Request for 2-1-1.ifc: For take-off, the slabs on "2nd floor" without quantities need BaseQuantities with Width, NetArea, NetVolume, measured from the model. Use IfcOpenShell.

First a look at what the model holds.

```python
import ifcopenshell
import ifcopenshell.util.element
import ifcopenshell.util.unit

model = ifcopenshell.open("2-1-1.ifc")
print(model.schema)
for unit_type in ("LENGTHUNIT", "AREAUNIT", "VOLUMEUNIT"):
    print(unit_type, ifcopenshell.util.unit.calculate_unit_scale(model, unit_type))
storey = next(s for s in model.by_type("IfcBuildingStorey") if s.Name == "2nd floor")
slabs = [e for e in ifcopenshell.util.element.get_decomposition(storey) if e.is_a("IfcSlab")]
for e in sorted(slabs, key=lambda e: e.id()):
    print(e.id(), e.is_a(), e.Name, list(ifcopenshell.util.element.get_psets(e, qtos_only=True)), sep=" | ")
```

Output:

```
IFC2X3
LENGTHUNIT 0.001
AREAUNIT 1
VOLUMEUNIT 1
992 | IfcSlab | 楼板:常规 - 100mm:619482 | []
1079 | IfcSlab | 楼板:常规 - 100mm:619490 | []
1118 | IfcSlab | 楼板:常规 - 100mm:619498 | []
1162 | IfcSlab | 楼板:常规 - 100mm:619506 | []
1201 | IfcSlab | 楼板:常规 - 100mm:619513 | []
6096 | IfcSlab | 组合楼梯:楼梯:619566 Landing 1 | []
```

```python
import ifcopenshell
import ifcopenshell.api.pset
import ifcopenshell.geom
import ifcopenshell.util.element
import ifcopenshell.util.shape
import ifcopenshell.util.unit

model = ifcopenshell.open("2-1-1.ifc")
unit_scale = ifcopenshell.util.unit.calculate_unit_scale(model)
area_scale = ifcopenshell.util.unit.calculate_unit_scale(model, "AREAUNIT")
volume_scale = ifcopenshell.util.unit.calculate_unit_scale(model, "VOLUMEUNIT")
settings = ifcopenshell.geom.settings()

storey = next(s for s in model.by_type("IfcBuildingStorey") if s.Name == "2nd floor")
slabs = [e for e in ifcopenshell.util.element.get_decomposition(storey) if e.is_a("IfcSlab")]

for e in sorted(slabs, key=lambda e: e.id()):
    if ifcopenshell.util.element.get_psets(e, qtos_only=True, should_inherit=False):
        continue
    # Geometry comes back in metres, in the element's own axes.
    shape = ifcopenshell.geom.create_shape(settings, e)
    values = {
        "Width": ifcopenshell.util.shape.get_z(shape.geometry) / unit_scale,
        "NetArea": ifcopenshell.util.shape.get_footprint_area(shape.geometry) / area_scale,
        "NetVolume": ifcopenshell.util.shape.get_volume(shape.geometry) / volume_scale,
    }
    qto = ifcopenshell.api.pset.add_qto(model, product=e, name="BaseQuantities")
    ifcopenshell.api.pset.edit_qto(model, qto=qto, properties=values)
    print(e.id(), {k: round(v, 3) for k, v in values.items()})

model.write("2-1-1_updated.ifc")
```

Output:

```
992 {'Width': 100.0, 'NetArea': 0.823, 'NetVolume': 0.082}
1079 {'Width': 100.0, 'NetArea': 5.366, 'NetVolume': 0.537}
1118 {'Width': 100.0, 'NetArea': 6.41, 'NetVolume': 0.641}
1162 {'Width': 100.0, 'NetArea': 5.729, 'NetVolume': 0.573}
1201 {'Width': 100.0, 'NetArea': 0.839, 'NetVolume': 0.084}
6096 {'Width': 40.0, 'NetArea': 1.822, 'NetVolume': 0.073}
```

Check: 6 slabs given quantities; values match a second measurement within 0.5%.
